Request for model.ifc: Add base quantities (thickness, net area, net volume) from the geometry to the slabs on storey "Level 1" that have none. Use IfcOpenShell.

First a look at what the model holds.

```python
import ifcopenshell
import ifcopenshell.util.element
import ifcopenshell.util.unit

model = ifcopenshell.open("model.ifc")
print(model.schema)
for unit_type in ("LENGTHUNIT", "AREAUNIT", "VOLUMEUNIT"):
    print(unit_type, ifcopenshell.util.unit.calculate_unit_scale(model, unit_type))
storey = next(s for s in model.by_type("IfcBuildingStorey") if s.Name == "Level 1")
slabs = [e for e in ifcopenshell.util.element.get_decomposition(storey) if e.is_a("IfcSlab")]
for e in sorted(slabs, key=lambda e: e.id()):
    print(e.id(), e.is_a(), e.Name, list(ifcopenshell.util.element.get_psets(e, qtos_only=True)), sep=" | ")
```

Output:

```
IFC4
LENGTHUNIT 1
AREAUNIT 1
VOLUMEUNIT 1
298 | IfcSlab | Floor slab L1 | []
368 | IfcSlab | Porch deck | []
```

```python
import ifcopenshell
import ifcopenshell.api.pset
import ifcopenshell.geom
import ifcopenshell.util.element
import ifcopenshell.util.shape
import ifcopenshell.util.unit

model = ifcopenshell.open("model.ifc")
unit_scale = ifcopenshell.util.unit.calculate_unit_scale(model)
area_scale = ifcopenshell.util.unit.calculate_unit_scale(model, "AREAUNIT")
volume_scale = ifcopenshell.util.unit.calculate_unit_scale(model, "VOLUMEUNIT")
settings = ifcopenshell.geom.settings()

storey = next(s for s in model.by_type("IfcBuildingStorey") if s.Name == "Level 1")
slabs = [e for e in ifcopenshell.util.element.get_decomposition(storey) if e.is_a("IfcSlab")]

for e in sorted(slabs, key=lambda e: e.id()):
    if ifcopenshell.util.element.get_psets(e, qtos_only=True, should_inherit=False):
        continue
    # Geometry comes back in metres, in the element's own axes.
    shape = ifcopenshell.geom.create_shape(settings, e)
    values = {
        "Width": ifcopenshell.util.shape.get_z(shape.geometry) / unit_scale,
        "NetArea": ifcopenshell.util.shape.get_footprint_area(shape.geometry) / area_scale,
        "NetVolume": ifcopenshell.util.shape.get_volume(shape.geometry) / volume_scale,
    }
    qto = ifcopenshell.api.pset.add_qto(model, product=e, name="Qto_SlabBaseQuantities")
    ifcopenshell.api.pset.edit_qto(model, qto=qto, properties=values)
    print(e.id(), {k: round(v, 3) for k, v in values.items()})

model.write("model_v2.ifc")
```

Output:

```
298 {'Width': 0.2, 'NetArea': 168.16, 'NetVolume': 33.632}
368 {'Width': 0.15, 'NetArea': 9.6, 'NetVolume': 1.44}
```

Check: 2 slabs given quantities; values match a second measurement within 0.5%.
